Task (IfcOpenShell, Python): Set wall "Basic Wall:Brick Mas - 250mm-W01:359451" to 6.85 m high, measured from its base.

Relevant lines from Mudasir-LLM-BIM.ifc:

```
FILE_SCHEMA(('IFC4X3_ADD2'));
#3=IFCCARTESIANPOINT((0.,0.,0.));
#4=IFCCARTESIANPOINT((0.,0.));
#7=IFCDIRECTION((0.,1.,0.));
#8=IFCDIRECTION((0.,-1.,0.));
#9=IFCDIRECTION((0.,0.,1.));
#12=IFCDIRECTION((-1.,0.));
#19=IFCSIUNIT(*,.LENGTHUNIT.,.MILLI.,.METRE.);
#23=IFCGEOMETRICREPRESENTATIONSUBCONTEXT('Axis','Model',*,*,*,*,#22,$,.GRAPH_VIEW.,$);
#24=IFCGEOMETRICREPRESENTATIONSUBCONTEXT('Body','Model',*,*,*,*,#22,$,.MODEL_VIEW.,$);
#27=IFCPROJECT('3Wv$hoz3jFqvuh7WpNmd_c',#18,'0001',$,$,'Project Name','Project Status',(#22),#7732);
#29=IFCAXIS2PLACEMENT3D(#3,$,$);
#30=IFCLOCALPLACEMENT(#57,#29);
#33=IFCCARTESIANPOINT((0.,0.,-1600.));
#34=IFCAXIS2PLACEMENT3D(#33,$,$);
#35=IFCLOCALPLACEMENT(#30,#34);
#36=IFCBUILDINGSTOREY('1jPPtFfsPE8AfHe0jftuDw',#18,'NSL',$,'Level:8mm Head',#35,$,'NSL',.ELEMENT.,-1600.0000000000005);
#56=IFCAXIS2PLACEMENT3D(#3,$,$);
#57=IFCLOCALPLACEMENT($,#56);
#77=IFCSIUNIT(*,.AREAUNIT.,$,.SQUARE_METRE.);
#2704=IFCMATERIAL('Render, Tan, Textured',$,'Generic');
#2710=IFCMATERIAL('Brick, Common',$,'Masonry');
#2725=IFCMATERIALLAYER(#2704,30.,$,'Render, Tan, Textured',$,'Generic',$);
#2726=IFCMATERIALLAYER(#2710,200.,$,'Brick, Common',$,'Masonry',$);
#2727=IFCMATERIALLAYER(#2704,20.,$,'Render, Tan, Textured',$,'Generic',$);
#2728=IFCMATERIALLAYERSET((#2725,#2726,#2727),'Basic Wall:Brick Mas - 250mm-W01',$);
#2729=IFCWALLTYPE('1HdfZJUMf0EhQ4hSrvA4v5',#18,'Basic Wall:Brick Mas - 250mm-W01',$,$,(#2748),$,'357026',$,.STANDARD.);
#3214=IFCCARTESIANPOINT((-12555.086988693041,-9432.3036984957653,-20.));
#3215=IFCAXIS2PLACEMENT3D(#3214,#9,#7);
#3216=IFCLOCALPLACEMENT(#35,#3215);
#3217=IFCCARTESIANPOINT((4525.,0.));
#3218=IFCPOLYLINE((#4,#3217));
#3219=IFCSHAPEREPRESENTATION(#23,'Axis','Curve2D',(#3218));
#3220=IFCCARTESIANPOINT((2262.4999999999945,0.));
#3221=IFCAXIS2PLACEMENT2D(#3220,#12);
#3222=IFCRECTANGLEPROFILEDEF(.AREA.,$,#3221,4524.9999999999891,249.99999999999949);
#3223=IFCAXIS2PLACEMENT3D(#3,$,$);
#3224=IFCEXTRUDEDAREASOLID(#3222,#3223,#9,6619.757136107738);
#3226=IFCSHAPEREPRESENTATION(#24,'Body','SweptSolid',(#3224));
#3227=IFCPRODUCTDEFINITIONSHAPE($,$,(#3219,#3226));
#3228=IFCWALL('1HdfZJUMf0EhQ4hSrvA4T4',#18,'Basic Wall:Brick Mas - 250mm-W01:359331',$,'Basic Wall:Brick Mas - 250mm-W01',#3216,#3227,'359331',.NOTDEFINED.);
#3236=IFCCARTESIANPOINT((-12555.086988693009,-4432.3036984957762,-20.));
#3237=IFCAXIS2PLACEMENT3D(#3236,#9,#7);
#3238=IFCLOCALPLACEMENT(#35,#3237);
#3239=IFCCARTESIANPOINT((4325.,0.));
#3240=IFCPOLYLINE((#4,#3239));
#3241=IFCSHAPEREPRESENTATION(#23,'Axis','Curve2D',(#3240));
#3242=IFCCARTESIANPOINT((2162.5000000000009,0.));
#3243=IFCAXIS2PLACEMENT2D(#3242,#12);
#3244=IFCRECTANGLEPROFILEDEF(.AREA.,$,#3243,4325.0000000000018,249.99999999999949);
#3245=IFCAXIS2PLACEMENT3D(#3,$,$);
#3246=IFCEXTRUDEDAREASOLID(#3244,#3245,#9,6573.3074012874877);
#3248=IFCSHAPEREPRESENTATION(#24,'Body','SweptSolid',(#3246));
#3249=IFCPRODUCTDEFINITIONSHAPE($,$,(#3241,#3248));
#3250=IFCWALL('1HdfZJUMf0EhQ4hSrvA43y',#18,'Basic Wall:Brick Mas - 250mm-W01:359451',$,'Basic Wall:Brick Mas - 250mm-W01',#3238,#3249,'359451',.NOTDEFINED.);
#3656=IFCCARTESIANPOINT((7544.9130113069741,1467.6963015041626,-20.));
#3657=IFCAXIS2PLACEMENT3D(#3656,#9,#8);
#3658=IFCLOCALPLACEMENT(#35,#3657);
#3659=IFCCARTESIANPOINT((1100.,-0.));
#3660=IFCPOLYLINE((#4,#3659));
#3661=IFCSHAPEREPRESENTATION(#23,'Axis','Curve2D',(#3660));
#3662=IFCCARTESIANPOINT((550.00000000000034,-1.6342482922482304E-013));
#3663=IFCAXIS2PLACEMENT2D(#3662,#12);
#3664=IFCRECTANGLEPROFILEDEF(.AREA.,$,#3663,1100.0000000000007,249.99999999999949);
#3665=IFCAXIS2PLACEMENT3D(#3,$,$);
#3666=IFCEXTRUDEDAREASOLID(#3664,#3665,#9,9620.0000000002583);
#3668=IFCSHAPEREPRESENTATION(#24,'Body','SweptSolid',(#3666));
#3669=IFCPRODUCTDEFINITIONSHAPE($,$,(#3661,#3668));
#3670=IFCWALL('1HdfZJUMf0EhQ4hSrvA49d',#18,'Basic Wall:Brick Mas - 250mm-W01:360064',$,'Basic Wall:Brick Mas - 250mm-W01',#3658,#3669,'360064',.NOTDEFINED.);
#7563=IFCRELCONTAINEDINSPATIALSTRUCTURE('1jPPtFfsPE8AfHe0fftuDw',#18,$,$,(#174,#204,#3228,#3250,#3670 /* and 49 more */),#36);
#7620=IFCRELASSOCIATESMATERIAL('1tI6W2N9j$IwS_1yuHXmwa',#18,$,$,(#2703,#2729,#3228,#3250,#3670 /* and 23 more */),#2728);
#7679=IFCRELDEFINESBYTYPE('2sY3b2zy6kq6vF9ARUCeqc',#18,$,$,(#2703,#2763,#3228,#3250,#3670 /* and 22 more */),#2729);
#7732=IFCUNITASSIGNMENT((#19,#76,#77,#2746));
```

```python
import ifcopenshell
import ifcopenshell.geom
import ifcopenshell.util.representation
import ifcopenshell.util.shape
import ifcopenshell.util.unit

model = ifcopenshell.open("Mudasir-LLM-BIM.ifc")
unit_scale = ifcopenshell.util.unit.calculate_unit_scale(model)
settings = ifcopenshell.geom.settings()


def volume(element):
    """Net volume in cubic metres, openings subtracted."""
    shape = ifcopenshell.geom.create_shape(settings, element)
    return ifcopenshell.util.shape.get_volume(shape.geometry)


wall = model.by_guid("1HdfZJUMf0EhQ4hSrvA43y")
before = volume(wall)

body = ifcopenshell.util.representation.get_representation(wall, "Model", "Body")
solid = body.Items[0]
old_height = solid.Depth
solid.Depth = 6.85 / unit_scale
after = volume(wall)

print(f"height {old_height:g} -> {solid.Depth:g}, volume {before:.3f} -> {after:.3f} m3")

model.write("Mudasir-LLM-BIM_v2.ifc")
```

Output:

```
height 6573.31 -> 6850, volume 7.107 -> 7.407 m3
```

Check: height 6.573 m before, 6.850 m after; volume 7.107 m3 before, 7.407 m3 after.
